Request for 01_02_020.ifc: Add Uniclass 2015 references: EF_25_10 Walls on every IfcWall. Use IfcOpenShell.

First a look at what the model holds.

```python
import ifcopenshell

model = ifcopenshell.open("01_02_020.ifc")
print(model.schema)
print("classifications:", [c.Name for c in model.by_type("IfcClassification")])
for ifc_class in ("IfcDoor", "IfcRoof", "IfcStair", "IfcWall", "IfcWindow"):
    print(ifc_class, len(model.by_type(ifc_class)))
```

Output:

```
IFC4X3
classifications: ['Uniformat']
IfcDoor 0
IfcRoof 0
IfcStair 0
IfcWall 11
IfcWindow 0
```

```python
import ifcopenshell
import ifcopenshell.api.classification

model = ifcopenshell.open("01_02_020.ifc")

system = ifcopenshell.api.classification.add_classification(model, classification="Uniclass 2015")

codes = {
    "IfcWall": ("EF_25_10", "Walls"),
}
for ifc_class, (code, name) in codes.items():
    products = model.by_type(ifc_class)
    ifcopenshell.api.classification.add_reference(
        model, products=products, classification=system, identification=code, name=name
    )
    print(code, len(products))

model.write("01_02_020-out.ifc")
```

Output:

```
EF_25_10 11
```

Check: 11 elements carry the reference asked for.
